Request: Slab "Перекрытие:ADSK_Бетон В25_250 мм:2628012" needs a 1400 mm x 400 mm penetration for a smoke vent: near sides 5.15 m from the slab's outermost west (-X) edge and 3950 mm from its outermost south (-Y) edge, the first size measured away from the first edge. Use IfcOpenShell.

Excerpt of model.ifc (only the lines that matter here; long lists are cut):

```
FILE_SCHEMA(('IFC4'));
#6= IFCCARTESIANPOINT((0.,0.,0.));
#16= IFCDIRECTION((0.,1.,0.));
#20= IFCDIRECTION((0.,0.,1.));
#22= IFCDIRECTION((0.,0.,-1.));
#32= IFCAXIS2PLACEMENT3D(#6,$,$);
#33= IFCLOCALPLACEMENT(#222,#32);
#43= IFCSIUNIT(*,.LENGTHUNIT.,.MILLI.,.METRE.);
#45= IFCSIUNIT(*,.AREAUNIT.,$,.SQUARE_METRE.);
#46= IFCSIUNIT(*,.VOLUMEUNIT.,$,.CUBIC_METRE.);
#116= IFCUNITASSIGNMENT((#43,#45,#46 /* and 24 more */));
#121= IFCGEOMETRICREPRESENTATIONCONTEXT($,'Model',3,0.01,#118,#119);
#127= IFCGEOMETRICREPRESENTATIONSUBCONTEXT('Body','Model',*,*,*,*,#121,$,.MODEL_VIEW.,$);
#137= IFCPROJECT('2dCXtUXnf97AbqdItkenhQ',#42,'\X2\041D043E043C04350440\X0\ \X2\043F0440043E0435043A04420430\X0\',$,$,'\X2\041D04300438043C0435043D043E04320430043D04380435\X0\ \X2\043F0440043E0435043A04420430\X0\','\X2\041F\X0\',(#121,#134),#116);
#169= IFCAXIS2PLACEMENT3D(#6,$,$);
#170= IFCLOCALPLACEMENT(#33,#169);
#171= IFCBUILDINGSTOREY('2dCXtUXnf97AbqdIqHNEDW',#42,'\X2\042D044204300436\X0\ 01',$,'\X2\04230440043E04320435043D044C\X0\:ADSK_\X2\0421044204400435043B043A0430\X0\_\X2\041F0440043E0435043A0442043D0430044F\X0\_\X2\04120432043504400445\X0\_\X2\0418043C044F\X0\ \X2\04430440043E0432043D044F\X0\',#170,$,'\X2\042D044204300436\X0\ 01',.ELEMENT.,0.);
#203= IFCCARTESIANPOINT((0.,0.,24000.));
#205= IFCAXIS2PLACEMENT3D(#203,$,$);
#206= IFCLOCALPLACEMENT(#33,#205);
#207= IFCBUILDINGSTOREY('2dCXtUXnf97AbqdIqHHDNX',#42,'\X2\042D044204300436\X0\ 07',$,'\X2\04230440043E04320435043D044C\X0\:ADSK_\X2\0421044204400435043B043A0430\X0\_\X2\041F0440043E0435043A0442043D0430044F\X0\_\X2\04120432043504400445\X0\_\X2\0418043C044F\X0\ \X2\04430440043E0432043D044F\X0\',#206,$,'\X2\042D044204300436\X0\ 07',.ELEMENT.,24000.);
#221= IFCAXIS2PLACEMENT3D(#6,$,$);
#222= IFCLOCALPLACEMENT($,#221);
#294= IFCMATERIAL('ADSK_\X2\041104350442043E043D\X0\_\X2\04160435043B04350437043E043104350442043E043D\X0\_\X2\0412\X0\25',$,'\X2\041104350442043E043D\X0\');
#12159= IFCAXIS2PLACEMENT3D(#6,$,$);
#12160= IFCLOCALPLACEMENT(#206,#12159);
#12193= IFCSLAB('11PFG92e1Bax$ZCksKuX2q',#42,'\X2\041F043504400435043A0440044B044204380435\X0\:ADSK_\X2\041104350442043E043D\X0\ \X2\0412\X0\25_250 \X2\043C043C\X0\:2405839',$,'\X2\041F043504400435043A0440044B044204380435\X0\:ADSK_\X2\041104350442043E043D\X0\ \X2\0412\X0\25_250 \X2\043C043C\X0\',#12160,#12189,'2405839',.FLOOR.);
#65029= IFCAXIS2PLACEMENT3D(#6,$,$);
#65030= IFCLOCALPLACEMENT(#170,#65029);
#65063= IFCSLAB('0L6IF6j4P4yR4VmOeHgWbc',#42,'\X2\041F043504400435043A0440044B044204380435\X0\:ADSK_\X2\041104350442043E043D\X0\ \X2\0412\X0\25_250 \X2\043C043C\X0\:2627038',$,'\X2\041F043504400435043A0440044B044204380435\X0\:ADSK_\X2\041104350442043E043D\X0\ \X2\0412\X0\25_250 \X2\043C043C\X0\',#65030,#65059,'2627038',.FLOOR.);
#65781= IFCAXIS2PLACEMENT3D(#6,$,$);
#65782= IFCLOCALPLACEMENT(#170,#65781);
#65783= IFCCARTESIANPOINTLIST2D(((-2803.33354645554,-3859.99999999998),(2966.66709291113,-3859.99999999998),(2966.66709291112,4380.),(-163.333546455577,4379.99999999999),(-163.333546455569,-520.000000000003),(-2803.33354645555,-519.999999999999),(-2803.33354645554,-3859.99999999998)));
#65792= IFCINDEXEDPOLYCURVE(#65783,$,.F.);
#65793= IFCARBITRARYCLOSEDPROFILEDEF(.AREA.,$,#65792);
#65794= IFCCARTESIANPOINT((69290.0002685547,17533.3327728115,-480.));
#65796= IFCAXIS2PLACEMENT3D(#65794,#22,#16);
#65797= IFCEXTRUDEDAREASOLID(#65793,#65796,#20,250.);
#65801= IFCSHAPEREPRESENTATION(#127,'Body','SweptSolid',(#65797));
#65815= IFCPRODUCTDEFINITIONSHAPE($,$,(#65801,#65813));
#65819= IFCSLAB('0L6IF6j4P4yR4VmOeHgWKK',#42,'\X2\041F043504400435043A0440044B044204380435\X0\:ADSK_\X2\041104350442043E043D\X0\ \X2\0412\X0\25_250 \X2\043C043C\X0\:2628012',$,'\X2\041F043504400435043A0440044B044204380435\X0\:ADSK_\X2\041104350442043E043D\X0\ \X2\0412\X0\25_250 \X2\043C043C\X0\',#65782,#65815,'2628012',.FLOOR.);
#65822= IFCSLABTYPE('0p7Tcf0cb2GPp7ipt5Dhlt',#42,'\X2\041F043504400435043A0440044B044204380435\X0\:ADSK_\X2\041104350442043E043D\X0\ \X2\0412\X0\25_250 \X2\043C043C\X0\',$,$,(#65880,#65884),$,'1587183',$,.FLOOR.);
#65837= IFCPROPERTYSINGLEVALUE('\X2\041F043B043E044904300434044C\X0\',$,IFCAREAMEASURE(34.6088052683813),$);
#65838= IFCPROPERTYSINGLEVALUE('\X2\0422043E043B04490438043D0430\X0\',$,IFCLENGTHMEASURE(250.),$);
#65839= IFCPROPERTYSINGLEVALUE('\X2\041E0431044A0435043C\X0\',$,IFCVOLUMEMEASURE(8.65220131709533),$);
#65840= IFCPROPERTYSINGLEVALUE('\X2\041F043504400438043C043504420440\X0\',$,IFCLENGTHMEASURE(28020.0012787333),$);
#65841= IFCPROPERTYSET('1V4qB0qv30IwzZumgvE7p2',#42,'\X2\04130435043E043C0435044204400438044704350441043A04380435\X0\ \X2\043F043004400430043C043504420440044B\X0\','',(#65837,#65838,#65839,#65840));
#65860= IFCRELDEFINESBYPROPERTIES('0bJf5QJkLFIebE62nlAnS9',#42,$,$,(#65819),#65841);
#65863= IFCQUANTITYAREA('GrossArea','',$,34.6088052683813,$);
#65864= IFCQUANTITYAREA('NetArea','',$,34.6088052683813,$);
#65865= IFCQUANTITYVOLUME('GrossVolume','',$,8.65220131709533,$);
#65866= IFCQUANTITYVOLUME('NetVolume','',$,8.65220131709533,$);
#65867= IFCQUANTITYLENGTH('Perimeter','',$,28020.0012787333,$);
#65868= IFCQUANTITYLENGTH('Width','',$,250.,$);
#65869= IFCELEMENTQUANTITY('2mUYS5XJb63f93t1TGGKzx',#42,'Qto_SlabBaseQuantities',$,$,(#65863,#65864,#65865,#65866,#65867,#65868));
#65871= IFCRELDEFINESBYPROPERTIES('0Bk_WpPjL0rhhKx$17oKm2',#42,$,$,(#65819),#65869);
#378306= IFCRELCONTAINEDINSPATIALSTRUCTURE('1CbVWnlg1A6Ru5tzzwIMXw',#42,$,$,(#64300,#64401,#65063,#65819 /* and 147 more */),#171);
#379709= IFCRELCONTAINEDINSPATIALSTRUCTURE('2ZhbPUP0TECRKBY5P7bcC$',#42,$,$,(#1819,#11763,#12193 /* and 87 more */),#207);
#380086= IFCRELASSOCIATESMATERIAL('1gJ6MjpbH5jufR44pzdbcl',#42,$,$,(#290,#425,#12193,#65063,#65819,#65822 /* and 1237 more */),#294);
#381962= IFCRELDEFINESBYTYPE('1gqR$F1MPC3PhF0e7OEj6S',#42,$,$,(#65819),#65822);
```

```python
import numpy as np
import ifcopenshell
import ifcopenshell.api.feature
import ifcopenshell.api.geometry
import ifcopenshell.api.pset
import ifcopenshell.api.root
import ifcopenshell.geom
import ifcopenshell.util.element
import ifcopenshell.util.placement
import ifcopenshell.util.representation
import ifcopenshell.util.shape
import ifcopenshell.util.unit

model = ifcopenshell.open("model.ifc")
unit_scale = ifcopenshell.util.unit.calculate_unit_scale(model)
area_scale = ifcopenshell.util.unit.calculate_unit_scale(model, "AREAUNIT")
volume_scale = ifcopenshell.util.unit.calculate_unit_scale(model, "VOLUMEUNIT")
settings = ifcopenshell.geom.settings()


def volume(element):
    """Net volume in cubic metres, openings subtracted."""
    shape = ifcopenshell.geom.create_shape(settings, element)
    return ifcopenshell.util.shape.get_volume(shape.geometry)


slab = model.by_id(65819)
before = volume(slab)

# Extent in the slab's own axes, in metres. The edges named are its -X and -Y sides.
slab_shape = ifcopenshell.geom.create_shape(settings, slab)
vertices = ifcopenshell.util.shape.get_vertices(slab_shape.geometry)
x_min, y_min, bottom = vertices.min(axis=0)
top = vertices[:, 2].max()

opening = ifcopenshell.api.root.create_entity(model, ifc_class="IfcOpeningElement", name="Smoke vent opening", predefined_type="OPENING")
context = ifcopenshell.util.representation.get_context(model, "Model", "Body", "MODEL_VIEW")
width, depth = 1.4, 0.4
outline = [(0.0, 0.0), (width, 0.0), (width, depth), (0.0, depth), (0.0, 0.0)]
# Overshoot both faces by 50 mm so the cut is clean.
shape = ifcopenshell.api.geometry.add_slab_representation(
    model, context=context, depth=top - bottom + 0.1, polyline=outline
)
ifcopenshell.api.geometry.assign_representation(model, product=opening, representation=shape)

matrix = ifcopenshell.util.placement.get_local_placement(slab.ObjectPlacement)
matrix[:, 3] = matrix @ np.append(np.array([x_min + 5.15, y_min + 3.95, bottom - 0.05]) / unit_scale, 1.0)
ifcopenshell.api.geometry.edit_object_placement(model, product=opening, matrix=matrix, is_si=False)
ifcopenshell.api.feature.add_feature(model, feature=opening, element=slab)

after = volume(slab)

# Update the slab's stored quantities.
pset = model.by_id(ifcopenshell.util.element.get_pset(slab, "Геометрические параметры", should_inherit=False)["id"])
ifcopenshell.api.pset.edit_pset(model, pset=pset, properties={
    "Площадь": model.create_entity("IfcAreaMeasure", after / (top - bottom) / area_scale),
    "Объем": model.create_entity("IfcVolumeMeasure", after / volume_scale),
})
qto = model.by_id(ifcopenshell.util.element.get_pset(slab, "Qto_SlabBaseQuantities", should_inherit=False)["id"])
ifcopenshell.api.pset.edit_qto(model, qto=qto, properties={
    "NetArea": after / (top - bottom) / area_scale,
    "NetVolume": after / volume_scale,
})

print(f"slab volume {before:.3f} -> {after:.3f} m3")

model.write("model_rev.ifc")
```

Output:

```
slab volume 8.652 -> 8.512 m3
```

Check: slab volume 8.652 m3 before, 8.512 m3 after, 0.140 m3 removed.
